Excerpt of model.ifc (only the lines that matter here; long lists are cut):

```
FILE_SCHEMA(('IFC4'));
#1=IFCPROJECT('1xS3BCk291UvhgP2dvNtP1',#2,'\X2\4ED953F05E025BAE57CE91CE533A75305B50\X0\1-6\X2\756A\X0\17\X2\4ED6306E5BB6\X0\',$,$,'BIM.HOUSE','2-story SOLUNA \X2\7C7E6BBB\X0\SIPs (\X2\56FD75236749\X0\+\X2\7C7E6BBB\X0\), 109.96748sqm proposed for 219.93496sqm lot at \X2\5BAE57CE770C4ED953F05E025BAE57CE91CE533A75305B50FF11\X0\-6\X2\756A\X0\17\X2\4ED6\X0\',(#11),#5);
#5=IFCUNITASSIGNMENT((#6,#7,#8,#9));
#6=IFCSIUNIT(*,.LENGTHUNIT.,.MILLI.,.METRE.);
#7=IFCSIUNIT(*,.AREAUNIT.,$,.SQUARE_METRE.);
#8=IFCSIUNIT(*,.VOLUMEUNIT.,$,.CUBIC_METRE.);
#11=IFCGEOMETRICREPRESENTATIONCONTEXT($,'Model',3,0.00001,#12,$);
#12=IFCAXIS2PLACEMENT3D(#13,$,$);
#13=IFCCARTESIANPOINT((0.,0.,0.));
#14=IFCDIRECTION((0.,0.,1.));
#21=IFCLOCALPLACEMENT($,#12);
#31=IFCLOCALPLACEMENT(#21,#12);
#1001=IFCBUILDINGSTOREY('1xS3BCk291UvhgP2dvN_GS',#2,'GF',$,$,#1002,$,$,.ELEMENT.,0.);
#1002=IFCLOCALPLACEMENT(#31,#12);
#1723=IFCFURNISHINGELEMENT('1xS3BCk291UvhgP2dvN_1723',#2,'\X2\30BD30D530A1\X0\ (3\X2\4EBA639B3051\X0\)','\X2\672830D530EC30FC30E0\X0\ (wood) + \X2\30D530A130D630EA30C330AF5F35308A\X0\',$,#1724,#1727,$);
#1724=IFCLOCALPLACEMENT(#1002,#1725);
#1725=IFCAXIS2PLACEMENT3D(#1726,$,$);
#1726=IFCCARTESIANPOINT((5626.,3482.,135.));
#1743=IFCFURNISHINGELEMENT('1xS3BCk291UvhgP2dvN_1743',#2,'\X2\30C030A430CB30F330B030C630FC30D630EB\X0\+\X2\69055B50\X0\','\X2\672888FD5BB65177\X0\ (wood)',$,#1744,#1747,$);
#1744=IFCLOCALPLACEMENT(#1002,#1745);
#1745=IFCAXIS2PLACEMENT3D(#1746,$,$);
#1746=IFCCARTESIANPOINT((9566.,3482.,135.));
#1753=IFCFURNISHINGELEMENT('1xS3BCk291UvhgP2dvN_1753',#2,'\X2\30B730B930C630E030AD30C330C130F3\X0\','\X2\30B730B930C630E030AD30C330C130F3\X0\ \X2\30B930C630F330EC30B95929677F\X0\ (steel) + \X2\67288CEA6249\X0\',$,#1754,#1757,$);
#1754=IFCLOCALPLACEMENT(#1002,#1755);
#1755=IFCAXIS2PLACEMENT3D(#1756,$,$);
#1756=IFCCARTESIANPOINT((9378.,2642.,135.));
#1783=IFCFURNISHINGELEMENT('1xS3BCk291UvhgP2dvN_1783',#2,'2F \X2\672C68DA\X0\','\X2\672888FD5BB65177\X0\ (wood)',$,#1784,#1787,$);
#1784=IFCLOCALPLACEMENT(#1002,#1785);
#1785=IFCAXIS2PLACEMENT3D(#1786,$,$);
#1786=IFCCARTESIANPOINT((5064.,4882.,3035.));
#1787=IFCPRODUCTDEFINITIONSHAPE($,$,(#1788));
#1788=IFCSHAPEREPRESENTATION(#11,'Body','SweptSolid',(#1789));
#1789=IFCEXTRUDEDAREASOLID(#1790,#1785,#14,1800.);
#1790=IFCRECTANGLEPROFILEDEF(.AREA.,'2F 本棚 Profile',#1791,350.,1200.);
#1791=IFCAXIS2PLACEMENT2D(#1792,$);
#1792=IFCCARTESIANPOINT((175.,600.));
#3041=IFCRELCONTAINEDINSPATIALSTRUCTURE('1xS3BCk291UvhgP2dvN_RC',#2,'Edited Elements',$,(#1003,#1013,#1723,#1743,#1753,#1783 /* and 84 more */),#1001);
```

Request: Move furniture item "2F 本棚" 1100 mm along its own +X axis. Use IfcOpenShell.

```python
import ifcopenshell
import ifcopenshell.api.geometry
import ifcopenshell.util.placement
import ifcopenshell.util.unit

model = ifcopenshell.open("model.ifc")
unit_scale = ifcopenshell.util.unit.calculate_unit_scale(model)

item = model.by_guid("1xS3BCk291UvhgP2dvN_1783")
matrix = ifcopenshell.util.placement.get_local_placement(item.ObjectPlacement)
matrix[:3, 3] += matrix[:3, 0] * 1.1 / unit_scale
ifcopenshell.api.geometry.edit_object_placement(model, product=item, matrix=matrix, is_si=False)

print(ifcopenshell.util.placement.get_local_placement(item.ObjectPlacement).round(3) + 0.0)

model.write("model_updated.ifc")
```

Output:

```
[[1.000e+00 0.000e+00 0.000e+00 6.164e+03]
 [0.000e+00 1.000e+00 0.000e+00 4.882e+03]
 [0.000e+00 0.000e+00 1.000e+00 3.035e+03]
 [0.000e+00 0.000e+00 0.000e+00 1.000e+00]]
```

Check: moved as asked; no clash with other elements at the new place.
